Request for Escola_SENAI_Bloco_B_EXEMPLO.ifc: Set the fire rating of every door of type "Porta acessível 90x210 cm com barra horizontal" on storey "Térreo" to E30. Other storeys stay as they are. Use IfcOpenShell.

First a look at what the model holds.

```python
import ifcopenshell
import ifcopenshell.util.element

model = ifcopenshell.open("Escola_SENAI_Bloco_B_EXEMPLO.ifc")
print(model.schema)
storey = next(s for s in model.by_type("IfcBuildingStorey") if s.Name == "Térreo")
doors = [e for e in ifcopenshell.util.element.get_decomposition(storey) if e.is_a("IfcDoor")]
seen = {}
for e in doors:
    element_type = ifcopenshell.util.element.get_type(e)
    key = (element_type.Name if element_type != e and element_type else None, ifcopenshell.util.element.get_pset(e, "Pset_DoorCommon", "FireRating"))
    seen[key] = seen.get(key, 0) + 1
for (name, value), count in sorted(seen.items(), key=str):
    print(count, "x", name, "|", value)
```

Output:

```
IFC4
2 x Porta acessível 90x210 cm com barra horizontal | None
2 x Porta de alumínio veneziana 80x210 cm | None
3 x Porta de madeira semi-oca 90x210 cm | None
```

```python
import ifcopenshell
import ifcopenshell.api.pset
import ifcopenshell.util.element

model = ifcopenshell.open("Escola_SENAI_Bloco_B_EXEMPLO.ifc")

storey = next(s for s in model.by_type("IfcBuildingStorey") if s.Name == "Térreo")
doors = [e for e in ifcopenshell.util.element.get_decomposition(storey) if e.is_a("IfcDoor")]

count = 0
for e in doors:
    element_type = ifcopenshell.util.element.get_type(e)
    if element_type in (None, e) or element_type.Name != "Porta acessível 90x210 cm com barra horizontal":
        continue
    # add_pset returns the element's existing set when there is one.
    pset = ifcopenshell.api.pset.add_pset(model, product=e, name="Pset_DoorCommon")
    ifcopenshell.api.pset.edit_pset(model, pset=pset, properties={"FireRating": "E30"})
    count += 1

print(count, "doors updated")

model.write("Escola_SENAI_Bloco_B_EXEMPLO_v2.ifc")
```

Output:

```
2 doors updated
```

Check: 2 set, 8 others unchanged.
